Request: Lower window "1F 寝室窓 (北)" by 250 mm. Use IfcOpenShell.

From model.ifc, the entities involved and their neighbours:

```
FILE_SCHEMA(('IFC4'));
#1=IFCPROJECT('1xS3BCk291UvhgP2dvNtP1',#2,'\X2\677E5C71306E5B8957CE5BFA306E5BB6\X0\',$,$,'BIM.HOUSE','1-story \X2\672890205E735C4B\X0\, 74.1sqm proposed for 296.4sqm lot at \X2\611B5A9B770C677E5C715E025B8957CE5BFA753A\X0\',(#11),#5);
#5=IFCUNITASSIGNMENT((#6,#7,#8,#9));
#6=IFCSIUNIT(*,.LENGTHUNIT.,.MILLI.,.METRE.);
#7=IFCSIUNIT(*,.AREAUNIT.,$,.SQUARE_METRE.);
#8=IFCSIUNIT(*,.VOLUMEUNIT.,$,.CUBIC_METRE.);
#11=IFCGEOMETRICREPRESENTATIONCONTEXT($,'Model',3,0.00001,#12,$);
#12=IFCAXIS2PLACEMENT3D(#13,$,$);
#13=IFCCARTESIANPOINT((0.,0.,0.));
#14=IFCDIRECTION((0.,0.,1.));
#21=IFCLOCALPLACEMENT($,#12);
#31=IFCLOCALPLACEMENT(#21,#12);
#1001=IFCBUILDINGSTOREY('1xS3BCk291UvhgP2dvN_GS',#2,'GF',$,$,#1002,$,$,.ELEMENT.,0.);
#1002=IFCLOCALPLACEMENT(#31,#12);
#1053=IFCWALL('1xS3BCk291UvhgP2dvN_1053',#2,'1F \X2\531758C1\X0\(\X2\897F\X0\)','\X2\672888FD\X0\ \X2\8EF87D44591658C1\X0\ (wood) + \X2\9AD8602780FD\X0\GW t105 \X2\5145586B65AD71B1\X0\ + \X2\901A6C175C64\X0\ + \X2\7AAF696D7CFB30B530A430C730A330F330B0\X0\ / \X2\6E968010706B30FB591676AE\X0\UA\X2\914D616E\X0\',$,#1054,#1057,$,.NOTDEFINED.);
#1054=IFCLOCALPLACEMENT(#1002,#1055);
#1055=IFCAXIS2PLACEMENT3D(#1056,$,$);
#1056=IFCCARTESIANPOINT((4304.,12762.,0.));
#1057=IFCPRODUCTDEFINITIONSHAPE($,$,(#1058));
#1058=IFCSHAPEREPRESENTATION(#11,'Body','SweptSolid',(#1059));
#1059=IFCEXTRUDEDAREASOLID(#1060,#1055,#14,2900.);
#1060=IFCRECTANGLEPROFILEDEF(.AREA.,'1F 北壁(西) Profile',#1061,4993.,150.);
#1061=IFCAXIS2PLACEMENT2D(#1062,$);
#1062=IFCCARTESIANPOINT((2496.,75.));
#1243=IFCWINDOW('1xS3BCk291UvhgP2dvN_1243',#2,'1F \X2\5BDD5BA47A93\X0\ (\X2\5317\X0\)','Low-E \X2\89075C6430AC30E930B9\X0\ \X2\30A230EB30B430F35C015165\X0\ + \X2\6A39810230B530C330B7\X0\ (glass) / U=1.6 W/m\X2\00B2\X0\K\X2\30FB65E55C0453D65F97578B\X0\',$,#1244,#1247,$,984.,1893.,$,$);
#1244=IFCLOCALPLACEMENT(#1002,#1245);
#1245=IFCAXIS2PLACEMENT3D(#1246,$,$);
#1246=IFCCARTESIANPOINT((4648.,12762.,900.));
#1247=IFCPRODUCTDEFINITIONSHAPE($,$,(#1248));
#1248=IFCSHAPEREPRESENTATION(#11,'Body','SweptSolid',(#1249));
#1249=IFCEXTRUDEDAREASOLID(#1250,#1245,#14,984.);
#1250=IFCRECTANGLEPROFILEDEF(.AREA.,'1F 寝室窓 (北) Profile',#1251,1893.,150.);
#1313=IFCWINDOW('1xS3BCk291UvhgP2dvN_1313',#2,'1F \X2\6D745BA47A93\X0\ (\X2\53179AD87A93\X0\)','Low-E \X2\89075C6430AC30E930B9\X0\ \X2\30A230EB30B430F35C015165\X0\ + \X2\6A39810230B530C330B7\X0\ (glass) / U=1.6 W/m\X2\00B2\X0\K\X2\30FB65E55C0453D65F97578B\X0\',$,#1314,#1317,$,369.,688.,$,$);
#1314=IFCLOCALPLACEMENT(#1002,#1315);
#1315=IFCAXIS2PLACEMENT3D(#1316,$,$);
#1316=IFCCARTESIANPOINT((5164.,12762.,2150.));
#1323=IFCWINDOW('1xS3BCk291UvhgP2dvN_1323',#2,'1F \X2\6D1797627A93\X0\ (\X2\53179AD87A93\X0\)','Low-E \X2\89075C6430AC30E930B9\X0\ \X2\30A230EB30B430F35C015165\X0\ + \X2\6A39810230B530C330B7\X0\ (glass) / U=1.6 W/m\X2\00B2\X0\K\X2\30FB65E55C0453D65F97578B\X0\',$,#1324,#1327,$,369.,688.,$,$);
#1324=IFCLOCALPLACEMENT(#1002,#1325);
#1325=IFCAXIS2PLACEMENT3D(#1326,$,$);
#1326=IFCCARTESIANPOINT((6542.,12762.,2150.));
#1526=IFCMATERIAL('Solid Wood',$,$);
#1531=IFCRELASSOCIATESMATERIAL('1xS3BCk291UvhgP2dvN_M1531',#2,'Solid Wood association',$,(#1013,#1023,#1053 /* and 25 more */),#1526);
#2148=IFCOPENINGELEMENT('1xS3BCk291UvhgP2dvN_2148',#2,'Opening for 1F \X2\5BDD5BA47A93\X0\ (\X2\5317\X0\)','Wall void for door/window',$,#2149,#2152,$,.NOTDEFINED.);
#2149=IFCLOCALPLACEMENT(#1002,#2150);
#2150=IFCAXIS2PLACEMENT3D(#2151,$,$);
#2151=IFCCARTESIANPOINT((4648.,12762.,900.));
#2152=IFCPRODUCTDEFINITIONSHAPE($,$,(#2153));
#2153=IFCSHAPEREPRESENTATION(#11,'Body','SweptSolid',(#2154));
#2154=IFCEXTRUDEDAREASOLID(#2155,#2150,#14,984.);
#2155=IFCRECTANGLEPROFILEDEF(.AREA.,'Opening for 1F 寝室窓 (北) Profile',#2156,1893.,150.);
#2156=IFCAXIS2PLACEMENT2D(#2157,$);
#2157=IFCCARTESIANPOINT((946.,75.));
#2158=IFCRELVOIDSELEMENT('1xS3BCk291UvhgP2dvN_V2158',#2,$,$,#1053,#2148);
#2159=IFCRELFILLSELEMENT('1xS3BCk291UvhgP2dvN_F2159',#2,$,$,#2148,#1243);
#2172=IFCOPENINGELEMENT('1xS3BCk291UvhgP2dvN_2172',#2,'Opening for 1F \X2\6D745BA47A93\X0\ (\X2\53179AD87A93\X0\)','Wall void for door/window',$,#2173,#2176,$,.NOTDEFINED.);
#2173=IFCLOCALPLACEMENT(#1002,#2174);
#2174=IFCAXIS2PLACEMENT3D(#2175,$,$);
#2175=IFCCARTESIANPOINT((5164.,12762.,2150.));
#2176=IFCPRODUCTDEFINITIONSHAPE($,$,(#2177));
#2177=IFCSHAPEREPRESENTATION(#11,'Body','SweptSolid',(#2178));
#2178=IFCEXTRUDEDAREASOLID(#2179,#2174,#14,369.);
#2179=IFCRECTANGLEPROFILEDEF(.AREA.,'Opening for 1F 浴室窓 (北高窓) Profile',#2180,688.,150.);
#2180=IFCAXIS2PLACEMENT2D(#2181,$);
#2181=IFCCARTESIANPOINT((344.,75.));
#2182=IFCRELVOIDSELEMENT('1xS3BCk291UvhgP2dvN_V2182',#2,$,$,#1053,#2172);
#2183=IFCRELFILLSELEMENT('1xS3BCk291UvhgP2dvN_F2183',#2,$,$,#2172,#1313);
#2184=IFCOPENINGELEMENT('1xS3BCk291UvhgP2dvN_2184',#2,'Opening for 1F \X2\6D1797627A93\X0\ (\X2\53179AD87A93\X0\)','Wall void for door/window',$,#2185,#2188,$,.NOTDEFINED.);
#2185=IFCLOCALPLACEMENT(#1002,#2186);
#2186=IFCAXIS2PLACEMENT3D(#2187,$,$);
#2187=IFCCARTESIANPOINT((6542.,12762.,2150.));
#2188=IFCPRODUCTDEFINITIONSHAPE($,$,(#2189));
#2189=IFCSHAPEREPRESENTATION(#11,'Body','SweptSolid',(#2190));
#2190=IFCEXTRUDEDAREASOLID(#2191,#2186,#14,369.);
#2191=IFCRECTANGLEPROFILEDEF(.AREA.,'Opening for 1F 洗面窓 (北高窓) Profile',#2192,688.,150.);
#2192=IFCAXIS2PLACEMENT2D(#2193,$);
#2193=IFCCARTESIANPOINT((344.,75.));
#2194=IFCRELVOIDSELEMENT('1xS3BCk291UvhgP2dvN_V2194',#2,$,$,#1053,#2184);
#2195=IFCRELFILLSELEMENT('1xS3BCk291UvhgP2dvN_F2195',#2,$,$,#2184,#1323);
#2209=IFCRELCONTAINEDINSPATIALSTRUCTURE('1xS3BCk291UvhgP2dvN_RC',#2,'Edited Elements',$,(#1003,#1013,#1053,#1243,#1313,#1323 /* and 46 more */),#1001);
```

```python
import numpy as np
import ifcopenshell
import ifcopenshell.api.geometry
import ifcopenshell.util.placement
import ifcopenshell.util.unit

model = ifcopenshell.open("model.ifc")
unit_scale = ifcopenshell.util.unit.calculate_unit_scale(model)

window = model.by_id(1243)
opening = window.FillsVoids[0].RelatingOpeningElement
dz = -0.25 / unit_scale

shift = np.array([0.0, 0.0, dz])
# The window is not placed relative to its opening, so move both.
for product in (opening, window):
    matrix = ifcopenshell.util.placement.get_local_placement(product.ObjectPlacement)
    matrix[:3, 3] += shift
    ifcopenshell.api.geometry.edit_object_placement(model, product=product, matrix=matrix, is_si=False)

print(f"moved by {dz * unit_scale:+.3f} m")

model.write("model_edited.ifc")
```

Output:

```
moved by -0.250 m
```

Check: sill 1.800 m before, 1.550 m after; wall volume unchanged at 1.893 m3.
